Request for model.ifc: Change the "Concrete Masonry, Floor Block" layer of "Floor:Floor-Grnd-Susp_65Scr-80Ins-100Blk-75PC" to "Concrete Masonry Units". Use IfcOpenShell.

First a look at what the model holds.

```python
import ifcopenshell
import ifcopenshell.util.element

model = ifcopenshell.open("model.ifc")
print(model.schema)
for layer_set in model.by_type("IfcMaterialLayerSet"):
    if layer_set.LayerSetName == "Floor:Floor-Grnd-Susp_65Scr-80Ins-100Blk-75PC":
        for layer in layer_set.MaterialLayers:
            print(layer.id(), layer.Material and layer.Material.Name, layer.LayerThickness, sep=" | ")
        print(len(ifcopenshell.util.element.get_elements_by_material(model, layer_set)), "elements and types use it")
print(sorted(m.Name for m in model.by_type("IfcMaterial") if m.Name)[:60])
```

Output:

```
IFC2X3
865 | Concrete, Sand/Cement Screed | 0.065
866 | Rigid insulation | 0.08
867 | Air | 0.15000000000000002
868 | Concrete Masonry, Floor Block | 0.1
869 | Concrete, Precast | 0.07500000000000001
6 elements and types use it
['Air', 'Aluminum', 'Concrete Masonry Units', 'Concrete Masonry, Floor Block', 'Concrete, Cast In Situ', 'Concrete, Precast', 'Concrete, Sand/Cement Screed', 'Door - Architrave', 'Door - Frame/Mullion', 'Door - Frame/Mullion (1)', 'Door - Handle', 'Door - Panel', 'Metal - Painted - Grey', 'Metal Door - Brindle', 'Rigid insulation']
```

```python
import ifcopenshell
import ifcopenshell.api.material

model = ifcopenshell.open("model.ifc")

layer_set = next(s for s in model.by_type("IfcMaterialLayerSet") if s.LayerSetName == "Floor:Floor-Grnd-Susp_65Scr-80Ins-100Blk-75PC")
layer = next(l for l in layer_set.MaterialLayers if l.Material and l.Material.Name == "Concrete Masonry, Floor Block")
material = next(m for m in model.by_type("IfcMaterial") if m.Name == "Concrete Masonry Units")

# Point this one layer at the other material; renaming the old one would change it everywhere.
ifcopenshell.api.material.edit_layer(model, layer=layer, attributes={}, material=material)

print([l.Material.Name if l.Material else None for l in layer_set.MaterialLayers])

model.write("model_updated.ifc")
```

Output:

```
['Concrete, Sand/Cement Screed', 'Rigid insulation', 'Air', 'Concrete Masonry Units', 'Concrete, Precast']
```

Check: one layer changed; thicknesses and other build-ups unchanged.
